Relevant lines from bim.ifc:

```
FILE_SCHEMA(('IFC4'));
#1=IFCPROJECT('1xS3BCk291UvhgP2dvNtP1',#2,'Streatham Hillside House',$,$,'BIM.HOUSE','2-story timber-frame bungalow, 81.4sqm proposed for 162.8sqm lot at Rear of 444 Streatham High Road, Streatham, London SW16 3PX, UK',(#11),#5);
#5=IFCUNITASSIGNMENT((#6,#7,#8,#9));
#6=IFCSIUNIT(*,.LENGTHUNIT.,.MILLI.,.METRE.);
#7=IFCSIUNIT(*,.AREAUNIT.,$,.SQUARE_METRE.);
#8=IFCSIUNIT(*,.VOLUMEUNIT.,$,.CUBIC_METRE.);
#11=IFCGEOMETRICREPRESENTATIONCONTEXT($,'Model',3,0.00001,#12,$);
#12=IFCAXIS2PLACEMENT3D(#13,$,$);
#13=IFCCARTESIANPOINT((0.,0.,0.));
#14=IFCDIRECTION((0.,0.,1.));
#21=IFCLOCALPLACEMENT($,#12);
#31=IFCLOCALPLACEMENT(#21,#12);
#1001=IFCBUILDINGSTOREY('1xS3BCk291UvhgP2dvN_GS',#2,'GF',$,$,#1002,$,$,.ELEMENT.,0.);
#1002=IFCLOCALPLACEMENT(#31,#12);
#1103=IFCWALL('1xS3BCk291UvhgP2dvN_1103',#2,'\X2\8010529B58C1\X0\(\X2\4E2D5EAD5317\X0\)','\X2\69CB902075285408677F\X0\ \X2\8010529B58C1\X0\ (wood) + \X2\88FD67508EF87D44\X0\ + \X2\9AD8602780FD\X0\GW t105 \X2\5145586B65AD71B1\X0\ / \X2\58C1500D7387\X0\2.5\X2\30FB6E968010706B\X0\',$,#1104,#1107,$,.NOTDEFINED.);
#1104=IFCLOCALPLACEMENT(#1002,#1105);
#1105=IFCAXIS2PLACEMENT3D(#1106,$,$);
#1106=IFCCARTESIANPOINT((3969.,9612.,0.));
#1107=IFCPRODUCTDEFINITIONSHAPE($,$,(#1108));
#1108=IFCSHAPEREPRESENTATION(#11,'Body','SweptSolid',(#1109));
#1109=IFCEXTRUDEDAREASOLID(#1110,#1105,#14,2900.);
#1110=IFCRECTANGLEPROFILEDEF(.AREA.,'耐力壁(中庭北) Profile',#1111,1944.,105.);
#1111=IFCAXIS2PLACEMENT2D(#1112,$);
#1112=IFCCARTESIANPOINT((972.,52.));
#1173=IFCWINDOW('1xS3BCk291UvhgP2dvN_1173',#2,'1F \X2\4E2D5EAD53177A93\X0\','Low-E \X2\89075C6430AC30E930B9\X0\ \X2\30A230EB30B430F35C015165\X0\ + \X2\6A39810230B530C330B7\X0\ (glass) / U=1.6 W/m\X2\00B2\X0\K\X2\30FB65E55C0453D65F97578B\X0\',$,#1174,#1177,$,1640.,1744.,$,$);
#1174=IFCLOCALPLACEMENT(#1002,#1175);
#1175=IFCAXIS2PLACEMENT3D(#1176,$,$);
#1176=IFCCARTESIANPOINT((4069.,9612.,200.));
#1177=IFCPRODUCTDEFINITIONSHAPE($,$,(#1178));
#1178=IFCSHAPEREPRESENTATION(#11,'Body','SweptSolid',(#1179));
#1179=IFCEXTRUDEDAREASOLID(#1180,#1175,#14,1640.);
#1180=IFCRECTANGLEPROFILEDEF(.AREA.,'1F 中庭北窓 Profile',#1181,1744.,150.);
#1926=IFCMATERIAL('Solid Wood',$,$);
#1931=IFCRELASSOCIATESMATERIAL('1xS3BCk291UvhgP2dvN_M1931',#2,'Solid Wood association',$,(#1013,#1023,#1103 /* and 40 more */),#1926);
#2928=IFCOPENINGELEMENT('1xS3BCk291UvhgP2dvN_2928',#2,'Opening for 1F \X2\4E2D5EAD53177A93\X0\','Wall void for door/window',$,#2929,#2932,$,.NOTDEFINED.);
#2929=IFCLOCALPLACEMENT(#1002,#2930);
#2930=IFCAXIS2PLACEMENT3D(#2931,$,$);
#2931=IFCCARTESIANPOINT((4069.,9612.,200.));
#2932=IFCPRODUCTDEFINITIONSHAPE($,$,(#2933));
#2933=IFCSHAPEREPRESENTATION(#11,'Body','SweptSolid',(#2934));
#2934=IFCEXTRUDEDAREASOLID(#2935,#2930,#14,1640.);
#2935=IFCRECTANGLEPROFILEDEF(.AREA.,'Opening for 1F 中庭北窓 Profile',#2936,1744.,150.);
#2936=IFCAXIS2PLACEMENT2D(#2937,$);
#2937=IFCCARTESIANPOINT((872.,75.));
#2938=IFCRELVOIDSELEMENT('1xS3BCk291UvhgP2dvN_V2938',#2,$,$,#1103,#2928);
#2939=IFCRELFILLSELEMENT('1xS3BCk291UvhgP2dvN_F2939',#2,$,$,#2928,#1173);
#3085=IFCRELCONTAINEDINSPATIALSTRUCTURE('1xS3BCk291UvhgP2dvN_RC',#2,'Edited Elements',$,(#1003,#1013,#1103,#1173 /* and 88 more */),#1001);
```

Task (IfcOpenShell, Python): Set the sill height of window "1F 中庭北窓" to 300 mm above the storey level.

```python
import numpy as np
import ifcopenshell
import ifcopenshell.api.geometry
import ifcopenshell.geom
import ifcopenshell.util.element
import ifcopenshell.util.placement
import ifcopenshell.util.shape
import ifcopenshell.util.unit

model = ifcopenshell.open("bim.ifc")
unit_scale = ifcopenshell.util.unit.calculate_unit_scale(model)

window = model.by_id(1173)
opening = window.FillsVoids[0].RelatingOpeningElement
storey = ifcopenshell.util.element.get_container(window, ifc_class="IfcBuildingStorey")
level = ifcopenshell.util.placement.get_local_placement(storey.ObjectPlacement)[2, 3]

# The opening's origin need not be at the sill, so measure its lowest point.
shape = ifcopenshell.geom.create_shape(ifcopenshell.geom.settings(), opening)
bottom = ifcopenshell.util.shape.get_shape_bottom_elevation(shape, shape.geometry) / unit_scale
dz = level + 300.0 - bottom

shift = np.array([0.0, 0.0, dz])
# The window is not placed relative to its opening, so move both.
for product in (opening, window):
    matrix = ifcopenshell.util.placement.get_local_placement(product.ObjectPlacement)
    matrix[:3, 3] += shift
    ifcopenshell.api.geometry.edit_object_placement(model, product=product, matrix=matrix, is_si=False)

print(f"moved by {dz * unit_scale:+.3f} m")

model.write("bim_rev.ifc")
```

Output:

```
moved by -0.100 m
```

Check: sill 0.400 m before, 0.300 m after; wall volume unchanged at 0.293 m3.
